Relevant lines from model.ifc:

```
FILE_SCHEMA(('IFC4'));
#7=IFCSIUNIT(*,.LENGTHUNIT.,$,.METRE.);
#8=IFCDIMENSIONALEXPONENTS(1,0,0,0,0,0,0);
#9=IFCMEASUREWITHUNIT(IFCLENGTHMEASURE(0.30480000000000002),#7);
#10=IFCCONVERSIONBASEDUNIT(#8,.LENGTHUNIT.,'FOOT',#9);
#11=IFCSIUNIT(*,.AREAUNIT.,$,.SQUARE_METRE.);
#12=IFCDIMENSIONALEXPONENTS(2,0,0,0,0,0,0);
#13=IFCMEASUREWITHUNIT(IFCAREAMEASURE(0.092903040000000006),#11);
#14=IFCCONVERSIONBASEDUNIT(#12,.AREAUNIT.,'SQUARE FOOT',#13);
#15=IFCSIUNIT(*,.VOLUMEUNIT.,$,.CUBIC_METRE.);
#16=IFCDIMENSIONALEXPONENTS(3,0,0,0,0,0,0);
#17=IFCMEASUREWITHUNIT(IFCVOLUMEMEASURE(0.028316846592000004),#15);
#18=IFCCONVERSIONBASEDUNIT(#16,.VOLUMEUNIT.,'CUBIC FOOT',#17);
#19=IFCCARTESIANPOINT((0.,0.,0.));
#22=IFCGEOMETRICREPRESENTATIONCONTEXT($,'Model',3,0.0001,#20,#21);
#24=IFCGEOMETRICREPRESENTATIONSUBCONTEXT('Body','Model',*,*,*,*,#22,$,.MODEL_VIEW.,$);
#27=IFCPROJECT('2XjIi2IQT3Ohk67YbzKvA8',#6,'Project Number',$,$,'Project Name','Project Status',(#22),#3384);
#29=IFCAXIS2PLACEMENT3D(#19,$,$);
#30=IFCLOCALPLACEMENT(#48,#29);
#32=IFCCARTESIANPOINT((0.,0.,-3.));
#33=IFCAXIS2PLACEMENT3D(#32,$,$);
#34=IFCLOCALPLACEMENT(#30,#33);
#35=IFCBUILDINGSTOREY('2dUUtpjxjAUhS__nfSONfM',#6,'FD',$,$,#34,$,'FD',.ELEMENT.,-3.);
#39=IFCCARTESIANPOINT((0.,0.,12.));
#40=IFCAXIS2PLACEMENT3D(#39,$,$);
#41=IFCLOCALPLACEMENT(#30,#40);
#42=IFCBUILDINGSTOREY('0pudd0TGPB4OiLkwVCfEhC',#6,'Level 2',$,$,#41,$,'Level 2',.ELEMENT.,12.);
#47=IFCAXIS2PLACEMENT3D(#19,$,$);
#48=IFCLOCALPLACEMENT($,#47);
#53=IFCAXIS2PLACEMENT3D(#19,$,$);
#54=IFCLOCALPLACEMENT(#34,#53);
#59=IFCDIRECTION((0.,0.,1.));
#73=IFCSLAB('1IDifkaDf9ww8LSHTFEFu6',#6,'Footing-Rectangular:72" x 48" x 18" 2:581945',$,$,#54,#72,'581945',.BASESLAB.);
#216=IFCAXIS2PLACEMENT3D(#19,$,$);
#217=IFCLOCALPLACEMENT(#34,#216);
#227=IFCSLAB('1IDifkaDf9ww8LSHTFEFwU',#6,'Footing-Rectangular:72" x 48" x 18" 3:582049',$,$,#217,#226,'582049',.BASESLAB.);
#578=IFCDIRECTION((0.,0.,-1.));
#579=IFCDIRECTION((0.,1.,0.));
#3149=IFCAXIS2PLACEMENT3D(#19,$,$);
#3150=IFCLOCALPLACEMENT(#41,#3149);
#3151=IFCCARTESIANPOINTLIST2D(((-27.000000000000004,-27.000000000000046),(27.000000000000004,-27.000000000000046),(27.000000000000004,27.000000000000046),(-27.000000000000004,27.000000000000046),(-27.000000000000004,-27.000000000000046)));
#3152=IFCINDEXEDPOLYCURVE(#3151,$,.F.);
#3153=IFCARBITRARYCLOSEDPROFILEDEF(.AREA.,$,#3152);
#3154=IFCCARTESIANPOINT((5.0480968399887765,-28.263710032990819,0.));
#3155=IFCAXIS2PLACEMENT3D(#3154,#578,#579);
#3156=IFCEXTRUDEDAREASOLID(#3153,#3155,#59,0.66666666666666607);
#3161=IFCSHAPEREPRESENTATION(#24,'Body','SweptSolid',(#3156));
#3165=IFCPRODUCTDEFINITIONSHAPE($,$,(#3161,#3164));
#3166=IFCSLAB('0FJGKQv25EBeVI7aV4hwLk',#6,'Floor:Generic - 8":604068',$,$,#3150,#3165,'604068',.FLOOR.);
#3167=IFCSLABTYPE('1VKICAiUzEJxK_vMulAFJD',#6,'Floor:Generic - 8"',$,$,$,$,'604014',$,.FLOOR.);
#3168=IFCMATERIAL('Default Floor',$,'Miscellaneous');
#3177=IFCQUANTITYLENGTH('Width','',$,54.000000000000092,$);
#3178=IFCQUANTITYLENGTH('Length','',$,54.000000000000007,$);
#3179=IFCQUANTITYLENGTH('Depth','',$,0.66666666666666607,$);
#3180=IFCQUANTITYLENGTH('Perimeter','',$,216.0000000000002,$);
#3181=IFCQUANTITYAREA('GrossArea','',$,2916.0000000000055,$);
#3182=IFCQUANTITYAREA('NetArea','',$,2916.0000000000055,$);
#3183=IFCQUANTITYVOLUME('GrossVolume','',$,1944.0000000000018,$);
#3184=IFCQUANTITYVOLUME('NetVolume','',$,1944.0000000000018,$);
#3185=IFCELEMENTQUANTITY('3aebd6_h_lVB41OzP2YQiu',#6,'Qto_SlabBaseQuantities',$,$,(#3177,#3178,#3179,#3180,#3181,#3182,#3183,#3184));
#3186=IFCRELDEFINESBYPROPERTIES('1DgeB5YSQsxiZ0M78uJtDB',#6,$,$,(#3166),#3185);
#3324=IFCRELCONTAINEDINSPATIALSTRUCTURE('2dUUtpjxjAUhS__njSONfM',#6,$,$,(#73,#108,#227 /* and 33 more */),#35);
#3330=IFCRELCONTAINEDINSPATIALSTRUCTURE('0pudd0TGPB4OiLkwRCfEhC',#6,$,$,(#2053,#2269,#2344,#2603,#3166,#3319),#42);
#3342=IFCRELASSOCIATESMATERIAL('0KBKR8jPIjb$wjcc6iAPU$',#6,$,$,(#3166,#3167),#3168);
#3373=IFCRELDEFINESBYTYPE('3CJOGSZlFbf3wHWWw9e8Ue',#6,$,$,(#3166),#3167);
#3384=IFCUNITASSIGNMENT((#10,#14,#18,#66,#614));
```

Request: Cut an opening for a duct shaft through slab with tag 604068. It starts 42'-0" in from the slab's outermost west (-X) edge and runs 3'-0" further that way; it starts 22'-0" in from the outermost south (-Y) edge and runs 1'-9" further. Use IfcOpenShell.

```python
import numpy as np
import ifcopenshell
import ifcopenshell.api.feature
import ifcopenshell.api.geometry
import ifcopenshell.api.pset
import ifcopenshell.api.root
import ifcopenshell.geom
import ifcopenshell.util.element
import ifcopenshell.util.placement
import ifcopenshell.util.representation
import ifcopenshell.util.shape
import ifcopenshell.util.unit

model = ifcopenshell.open("model.ifc")
unit_scale = ifcopenshell.util.unit.calculate_unit_scale(model)
area_scale = ifcopenshell.util.unit.calculate_unit_scale(model, "AREAUNIT")
volume_scale = ifcopenshell.util.unit.calculate_unit_scale(model, "VOLUMEUNIT")
settings = ifcopenshell.geom.settings()


def volume(element):
    """Net volume in cubic metres, openings subtracted."""
    shape = ifcopenshell.geom.create_shape(settings, element)
    return ifcopenshell.util.shape.get_volume(shape.geometry)


slab = model.by_guid("0FJGKQv25EBeVI7aV4hwLk")
before = volume(slab)

# Extent in the slab's own axes, in metres. The edges named are its -X and -Y sides.
slab_shape = ifcopenshell.geom.create_shape(settings, slab)
vertices = ifcopenshell.util.shape.get_vertices(slab_shape.geometry)
x_min, y_min, bottom = vertices.min(axis=0)
top = vertices[:, 2].max()

opening = ifcopenshell.api.root.create_entity(model, ifc_class="IfcOpeningElement", name="Duct shaft opening", predefined_type="OPENING")
context = ifcopenshell.util.representation.get_context(model, "Model", "Body", "MODEL_VIEW")
width, depth = 0.9144, 0.5334
outline = [(0.0, 0.0), (width, 0.0), (width, depth), (0.0, depth), (0.0, 0.0)]
# Overshoot both faces by 50 mm so the cut is clean.
shape = ifcopenshell.api.geometry.add_slab_representation(
    model, context=context, depth=top - bottom + 0.1, polyline=outline
)
ifcopenshell.api.geometry.assign_representation(model, product=opening, representation=shape)

matrix = ifcopenshell.util.placement.get_local_placement(slab.ObjectPlacement)
matrix[:, 3] = matrix @ np.append(np.array([x_min + 12.8016, y_min + 6.7056, bottom - 0.05]) / unit_scale, 1.0)
ifcopenshell.api.geometry.edit_object_placement(model, product=opening, matrix=matrix, is_si=False)
ifcopenshell.api.feature.add_feature(model, feature=opening, element=slab)

after = volume(slab)

# Update the slab's stored quantities.
qto = model.by_id(ifcopenshell.util.element.get_pset(slab, "Qto_SlabBaseQuantities", should_inherit=False)["id"])
ifcopenshell.api.pset.edit_qto(model, qto=qto, properties={
    "NetArea": after / (top - bottom) / area_scale,
    "NetVolume": after / volume_scale,
})

print(f"slab volume {before:.3f} -> {after:.3f} m3")

model.write("model_updated.ifc")
```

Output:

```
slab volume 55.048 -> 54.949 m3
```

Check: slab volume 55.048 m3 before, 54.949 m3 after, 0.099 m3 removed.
